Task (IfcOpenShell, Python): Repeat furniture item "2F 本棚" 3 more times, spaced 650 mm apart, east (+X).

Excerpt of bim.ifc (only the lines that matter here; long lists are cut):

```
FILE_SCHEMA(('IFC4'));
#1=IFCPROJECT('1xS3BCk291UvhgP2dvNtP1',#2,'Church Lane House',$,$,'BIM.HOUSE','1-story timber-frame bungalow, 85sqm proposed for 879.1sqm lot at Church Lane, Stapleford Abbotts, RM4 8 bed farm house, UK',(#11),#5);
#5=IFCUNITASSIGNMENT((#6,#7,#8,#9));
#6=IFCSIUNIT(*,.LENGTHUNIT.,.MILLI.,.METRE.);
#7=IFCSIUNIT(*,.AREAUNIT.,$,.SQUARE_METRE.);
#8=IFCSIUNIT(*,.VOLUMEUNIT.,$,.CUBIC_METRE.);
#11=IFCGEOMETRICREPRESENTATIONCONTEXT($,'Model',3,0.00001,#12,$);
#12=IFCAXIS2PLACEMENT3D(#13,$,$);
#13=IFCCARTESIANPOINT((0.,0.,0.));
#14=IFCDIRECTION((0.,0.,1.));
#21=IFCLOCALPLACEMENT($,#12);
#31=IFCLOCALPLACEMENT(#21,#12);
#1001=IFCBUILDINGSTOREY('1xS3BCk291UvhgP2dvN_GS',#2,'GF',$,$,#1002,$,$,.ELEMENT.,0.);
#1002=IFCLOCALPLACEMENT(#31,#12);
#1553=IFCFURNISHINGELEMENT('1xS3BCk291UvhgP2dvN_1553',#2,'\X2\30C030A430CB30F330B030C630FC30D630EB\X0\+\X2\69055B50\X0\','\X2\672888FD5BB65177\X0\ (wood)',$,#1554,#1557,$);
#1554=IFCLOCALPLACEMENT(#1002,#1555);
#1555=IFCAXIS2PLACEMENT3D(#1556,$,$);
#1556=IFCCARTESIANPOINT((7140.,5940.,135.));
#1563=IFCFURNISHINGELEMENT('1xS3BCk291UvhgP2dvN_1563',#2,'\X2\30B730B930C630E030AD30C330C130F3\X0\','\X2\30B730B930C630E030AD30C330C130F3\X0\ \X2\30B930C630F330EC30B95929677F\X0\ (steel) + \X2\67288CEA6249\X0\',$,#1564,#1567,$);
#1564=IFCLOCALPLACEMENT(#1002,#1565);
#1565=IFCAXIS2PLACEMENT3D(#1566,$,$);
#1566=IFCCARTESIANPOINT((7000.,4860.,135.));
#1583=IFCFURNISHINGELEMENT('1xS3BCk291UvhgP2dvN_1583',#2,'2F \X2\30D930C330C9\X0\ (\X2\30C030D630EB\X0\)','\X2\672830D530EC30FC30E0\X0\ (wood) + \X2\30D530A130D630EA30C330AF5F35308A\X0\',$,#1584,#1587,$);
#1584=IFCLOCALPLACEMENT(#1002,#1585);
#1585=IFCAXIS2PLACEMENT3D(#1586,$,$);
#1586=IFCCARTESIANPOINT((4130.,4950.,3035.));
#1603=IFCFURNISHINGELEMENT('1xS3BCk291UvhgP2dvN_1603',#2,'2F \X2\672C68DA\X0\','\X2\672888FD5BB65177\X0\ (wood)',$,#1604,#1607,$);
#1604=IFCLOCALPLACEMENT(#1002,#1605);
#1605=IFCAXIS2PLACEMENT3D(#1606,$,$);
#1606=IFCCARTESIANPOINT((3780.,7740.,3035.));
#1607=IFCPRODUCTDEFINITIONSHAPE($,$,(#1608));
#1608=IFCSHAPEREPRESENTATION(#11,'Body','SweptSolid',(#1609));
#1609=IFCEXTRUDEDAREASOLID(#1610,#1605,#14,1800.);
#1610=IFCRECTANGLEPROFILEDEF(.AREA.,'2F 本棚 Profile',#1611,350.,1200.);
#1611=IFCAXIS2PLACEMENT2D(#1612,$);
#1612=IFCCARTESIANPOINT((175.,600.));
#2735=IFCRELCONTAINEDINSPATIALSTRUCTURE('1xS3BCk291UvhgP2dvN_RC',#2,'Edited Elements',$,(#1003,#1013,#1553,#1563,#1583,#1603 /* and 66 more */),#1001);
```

```python
import numpy as np
import ifcopenshell
import ifcopenshell.api.geometry
import ifcopenshell.api.root
import ifcopenshell.util.element
import ifcopenshell.util.placement
import ifcopenshell.util.unit

model = ifcopenshell.open("bim.ifc")
unit_scale = ifcopenshell.util.unit.calculate_unit_scale(model)


def reuse_history(source, copy):
    """copy_class also copies each property set's owner history, people and application; keep the originals."""
    for rel in copy.IsDefinedBy:
        if rel.is_a("IfcRelDefinesByProperties") and (history := rel.RelatingPropertyDefinition.OwnerHistory):
            rel.RelatingPropertyDefinition.OwnerHistory = source.OwnerHistory
            ifcopenshell.util.element.remove_deep2(model, history)


source = model.by_guid("1xS3BCk291UvhgP2dvN_1603")
base = ifcopenshell.util.placement.get_local_placement(source.ObjectPlacement)
step = np.array([1.0, 0.0, 0.0]) * 0.65 / unit_scale

for i in range(1, 4):
    copy = ifcopenshell.api.root.copy_class(model, product=source)
    copy.Representation = ifcopenshell.util.element.copy_deep(
        model, source.Representation, exclude=["IfcGeometricRepresentationContext", "IfcRepresentationMap"]
    )
    reuse_history(source, copy)
    matrix = base.copy()
    matrix[:3, 3] += i * step
    print("added at", matrix[:3, 3].round(3) + 0.0)
    ifcopenshell.api.geometry.edit_object_placement(model, product=copy, matrix=matrix, is_si=False)

model.write("bim-out.ifc")
```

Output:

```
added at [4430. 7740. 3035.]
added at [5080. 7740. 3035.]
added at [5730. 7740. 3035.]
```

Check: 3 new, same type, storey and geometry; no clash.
